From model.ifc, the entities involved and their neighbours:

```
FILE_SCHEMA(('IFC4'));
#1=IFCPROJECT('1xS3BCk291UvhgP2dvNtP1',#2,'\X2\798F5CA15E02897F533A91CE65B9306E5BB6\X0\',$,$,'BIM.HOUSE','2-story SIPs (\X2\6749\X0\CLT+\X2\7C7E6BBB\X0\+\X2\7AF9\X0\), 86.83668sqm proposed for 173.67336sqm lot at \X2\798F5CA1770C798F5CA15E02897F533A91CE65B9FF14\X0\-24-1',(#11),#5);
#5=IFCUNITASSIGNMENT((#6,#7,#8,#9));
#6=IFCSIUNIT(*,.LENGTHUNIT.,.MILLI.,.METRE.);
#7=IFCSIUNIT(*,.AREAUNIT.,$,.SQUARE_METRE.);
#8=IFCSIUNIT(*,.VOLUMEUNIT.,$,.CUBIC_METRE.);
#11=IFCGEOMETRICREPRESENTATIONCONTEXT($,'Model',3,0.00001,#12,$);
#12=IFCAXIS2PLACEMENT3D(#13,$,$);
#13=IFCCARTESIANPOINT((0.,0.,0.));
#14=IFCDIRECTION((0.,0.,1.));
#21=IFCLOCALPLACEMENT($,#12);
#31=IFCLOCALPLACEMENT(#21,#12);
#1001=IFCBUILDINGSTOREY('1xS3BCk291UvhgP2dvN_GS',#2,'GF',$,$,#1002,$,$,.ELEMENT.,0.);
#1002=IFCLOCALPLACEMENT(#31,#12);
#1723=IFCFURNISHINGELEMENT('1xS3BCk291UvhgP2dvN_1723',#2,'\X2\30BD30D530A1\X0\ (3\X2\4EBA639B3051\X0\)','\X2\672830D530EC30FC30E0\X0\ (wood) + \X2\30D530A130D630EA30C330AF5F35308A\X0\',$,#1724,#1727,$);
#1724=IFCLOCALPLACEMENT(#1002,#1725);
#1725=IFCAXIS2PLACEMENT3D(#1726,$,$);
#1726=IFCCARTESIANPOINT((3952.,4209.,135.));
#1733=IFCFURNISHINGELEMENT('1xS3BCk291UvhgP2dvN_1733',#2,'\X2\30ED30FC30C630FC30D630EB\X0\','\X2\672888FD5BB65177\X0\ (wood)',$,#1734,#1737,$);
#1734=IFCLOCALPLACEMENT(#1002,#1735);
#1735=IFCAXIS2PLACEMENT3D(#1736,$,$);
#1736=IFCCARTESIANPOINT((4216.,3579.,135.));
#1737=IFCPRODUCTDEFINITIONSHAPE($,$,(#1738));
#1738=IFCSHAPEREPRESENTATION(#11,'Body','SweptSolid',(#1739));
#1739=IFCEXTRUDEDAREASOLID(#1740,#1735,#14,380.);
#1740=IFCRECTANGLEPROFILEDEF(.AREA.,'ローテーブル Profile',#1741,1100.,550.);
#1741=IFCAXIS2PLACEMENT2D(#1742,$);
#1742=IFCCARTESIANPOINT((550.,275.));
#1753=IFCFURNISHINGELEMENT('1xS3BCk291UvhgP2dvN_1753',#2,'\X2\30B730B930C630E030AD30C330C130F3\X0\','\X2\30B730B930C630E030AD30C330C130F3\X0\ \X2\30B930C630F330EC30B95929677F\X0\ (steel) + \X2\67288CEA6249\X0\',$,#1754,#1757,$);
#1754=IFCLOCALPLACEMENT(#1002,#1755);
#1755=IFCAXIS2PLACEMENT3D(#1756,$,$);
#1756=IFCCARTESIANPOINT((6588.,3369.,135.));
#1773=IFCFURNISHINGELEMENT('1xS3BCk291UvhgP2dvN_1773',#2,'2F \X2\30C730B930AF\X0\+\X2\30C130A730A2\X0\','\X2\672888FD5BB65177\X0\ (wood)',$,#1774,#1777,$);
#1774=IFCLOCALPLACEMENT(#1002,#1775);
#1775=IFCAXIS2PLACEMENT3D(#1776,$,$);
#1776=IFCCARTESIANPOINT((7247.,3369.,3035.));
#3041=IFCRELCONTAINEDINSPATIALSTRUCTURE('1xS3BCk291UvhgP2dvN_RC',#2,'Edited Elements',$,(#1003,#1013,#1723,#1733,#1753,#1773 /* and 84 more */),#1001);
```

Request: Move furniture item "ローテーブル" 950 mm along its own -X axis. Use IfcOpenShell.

```python
import ifcopenshell
import ifcopenshell.api.geometry
import ifcopenshell.util.placement
import ifcopenshell.util.unit

model = ifcopenshell.open("model.ifc")
unit_scale = ifcopenshell.util.unit.calculate_unit_scale(model)

item = model.by_guid("1xS3BCk291UvhgP2dvN_1733")
matrix = ifcopenshell.util.placement.get_local_placement(item.ObjectPlacement)
matrix[:3, 3] -= matrix[:3, 0] * 0.95 / unit_scale
ifcopenshell.api.geometry.edit_object_placement(model, product=item, matrix=matrix, is_si=False)

print(ifcopenshell.util.placement.get_local_placement(item.ObjectPlacement).round(3) + 0.0)

model.write("model-out.ifc")
```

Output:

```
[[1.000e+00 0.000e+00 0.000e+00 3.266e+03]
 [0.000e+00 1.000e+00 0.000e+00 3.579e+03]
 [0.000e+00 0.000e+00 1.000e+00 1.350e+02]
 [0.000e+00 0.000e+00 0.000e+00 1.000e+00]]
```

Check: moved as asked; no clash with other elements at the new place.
